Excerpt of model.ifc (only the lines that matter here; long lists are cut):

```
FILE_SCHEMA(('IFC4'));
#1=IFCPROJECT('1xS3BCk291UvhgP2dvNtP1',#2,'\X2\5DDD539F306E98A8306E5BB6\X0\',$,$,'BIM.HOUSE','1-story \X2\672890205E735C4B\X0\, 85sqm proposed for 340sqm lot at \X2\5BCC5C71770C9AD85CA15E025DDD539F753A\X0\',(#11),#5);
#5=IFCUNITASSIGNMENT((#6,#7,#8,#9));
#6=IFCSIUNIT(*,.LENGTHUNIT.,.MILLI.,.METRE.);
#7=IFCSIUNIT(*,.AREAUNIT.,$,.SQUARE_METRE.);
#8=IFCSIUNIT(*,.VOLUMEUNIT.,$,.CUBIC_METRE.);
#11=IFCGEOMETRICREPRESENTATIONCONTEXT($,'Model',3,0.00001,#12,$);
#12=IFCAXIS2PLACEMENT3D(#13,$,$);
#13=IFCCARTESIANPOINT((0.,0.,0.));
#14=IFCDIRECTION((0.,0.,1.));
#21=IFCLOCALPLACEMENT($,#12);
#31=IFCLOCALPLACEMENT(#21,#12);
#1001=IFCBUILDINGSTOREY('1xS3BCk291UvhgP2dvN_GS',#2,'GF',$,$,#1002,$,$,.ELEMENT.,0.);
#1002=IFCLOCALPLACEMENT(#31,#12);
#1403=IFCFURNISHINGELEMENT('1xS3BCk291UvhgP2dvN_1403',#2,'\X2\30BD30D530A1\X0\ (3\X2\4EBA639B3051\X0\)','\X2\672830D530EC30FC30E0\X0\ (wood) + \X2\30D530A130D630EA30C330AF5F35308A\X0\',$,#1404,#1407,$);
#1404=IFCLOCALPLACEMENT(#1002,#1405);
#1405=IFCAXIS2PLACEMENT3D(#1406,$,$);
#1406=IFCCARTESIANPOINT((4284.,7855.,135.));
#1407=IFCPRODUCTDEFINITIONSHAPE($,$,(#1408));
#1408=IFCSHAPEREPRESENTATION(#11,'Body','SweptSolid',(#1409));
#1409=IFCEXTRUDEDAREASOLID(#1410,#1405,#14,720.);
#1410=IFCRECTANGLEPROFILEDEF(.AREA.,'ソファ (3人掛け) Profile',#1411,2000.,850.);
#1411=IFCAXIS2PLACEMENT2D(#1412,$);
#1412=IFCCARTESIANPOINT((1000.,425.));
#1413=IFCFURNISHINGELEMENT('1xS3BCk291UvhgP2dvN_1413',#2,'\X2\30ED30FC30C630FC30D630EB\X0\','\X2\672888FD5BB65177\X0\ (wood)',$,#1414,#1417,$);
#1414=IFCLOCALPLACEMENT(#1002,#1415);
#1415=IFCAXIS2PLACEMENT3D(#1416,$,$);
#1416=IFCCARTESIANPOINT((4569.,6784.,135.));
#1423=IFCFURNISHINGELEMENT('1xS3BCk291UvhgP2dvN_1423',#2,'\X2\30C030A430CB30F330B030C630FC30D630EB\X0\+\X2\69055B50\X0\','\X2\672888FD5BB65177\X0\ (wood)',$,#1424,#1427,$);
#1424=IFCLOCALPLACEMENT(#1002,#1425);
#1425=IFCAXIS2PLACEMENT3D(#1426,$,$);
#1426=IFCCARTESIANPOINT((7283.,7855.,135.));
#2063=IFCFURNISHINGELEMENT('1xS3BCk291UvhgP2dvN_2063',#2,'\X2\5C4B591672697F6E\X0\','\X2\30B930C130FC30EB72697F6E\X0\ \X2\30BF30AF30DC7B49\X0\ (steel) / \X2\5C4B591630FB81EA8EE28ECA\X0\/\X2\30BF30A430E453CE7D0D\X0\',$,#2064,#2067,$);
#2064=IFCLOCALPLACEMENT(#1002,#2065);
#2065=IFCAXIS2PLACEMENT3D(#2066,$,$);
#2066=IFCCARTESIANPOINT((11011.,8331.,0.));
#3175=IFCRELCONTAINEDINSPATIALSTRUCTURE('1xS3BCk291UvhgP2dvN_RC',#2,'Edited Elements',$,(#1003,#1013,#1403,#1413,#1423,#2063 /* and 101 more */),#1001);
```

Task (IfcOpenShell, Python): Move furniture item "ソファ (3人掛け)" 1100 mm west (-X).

```python
import ifcopenshell
import ifcopenshell.api.geometry
import ifcopenshell.util.placement
import ifcopenshell.util.unit

model = ifcopenshell.open("model.ifc")
unit_scale = ifcopenshell.util.unit.calculate_unit_scale(model)

item = model.by_guid("1xS3BCk291UvhgP2dvN_1403")
matrix = ifcopenshell.util.placement.get_local_placement(item.ObjectPlacement)
matrix[0, 3] -= 1.1 / unit_scale
ifcopenshell.api.geometry.edit_object_placement(model, product=item, matrix=matrix, is_si=False)

print(ifcopenshell.util.placement.get_local_placement(item.ObjectPlacement).round(3) + 0.0)

model.write("model_v2.ifc")
```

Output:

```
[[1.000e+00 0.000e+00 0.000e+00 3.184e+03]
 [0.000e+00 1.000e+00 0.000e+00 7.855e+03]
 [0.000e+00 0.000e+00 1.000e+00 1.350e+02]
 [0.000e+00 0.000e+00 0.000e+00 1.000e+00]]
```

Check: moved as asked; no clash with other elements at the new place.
